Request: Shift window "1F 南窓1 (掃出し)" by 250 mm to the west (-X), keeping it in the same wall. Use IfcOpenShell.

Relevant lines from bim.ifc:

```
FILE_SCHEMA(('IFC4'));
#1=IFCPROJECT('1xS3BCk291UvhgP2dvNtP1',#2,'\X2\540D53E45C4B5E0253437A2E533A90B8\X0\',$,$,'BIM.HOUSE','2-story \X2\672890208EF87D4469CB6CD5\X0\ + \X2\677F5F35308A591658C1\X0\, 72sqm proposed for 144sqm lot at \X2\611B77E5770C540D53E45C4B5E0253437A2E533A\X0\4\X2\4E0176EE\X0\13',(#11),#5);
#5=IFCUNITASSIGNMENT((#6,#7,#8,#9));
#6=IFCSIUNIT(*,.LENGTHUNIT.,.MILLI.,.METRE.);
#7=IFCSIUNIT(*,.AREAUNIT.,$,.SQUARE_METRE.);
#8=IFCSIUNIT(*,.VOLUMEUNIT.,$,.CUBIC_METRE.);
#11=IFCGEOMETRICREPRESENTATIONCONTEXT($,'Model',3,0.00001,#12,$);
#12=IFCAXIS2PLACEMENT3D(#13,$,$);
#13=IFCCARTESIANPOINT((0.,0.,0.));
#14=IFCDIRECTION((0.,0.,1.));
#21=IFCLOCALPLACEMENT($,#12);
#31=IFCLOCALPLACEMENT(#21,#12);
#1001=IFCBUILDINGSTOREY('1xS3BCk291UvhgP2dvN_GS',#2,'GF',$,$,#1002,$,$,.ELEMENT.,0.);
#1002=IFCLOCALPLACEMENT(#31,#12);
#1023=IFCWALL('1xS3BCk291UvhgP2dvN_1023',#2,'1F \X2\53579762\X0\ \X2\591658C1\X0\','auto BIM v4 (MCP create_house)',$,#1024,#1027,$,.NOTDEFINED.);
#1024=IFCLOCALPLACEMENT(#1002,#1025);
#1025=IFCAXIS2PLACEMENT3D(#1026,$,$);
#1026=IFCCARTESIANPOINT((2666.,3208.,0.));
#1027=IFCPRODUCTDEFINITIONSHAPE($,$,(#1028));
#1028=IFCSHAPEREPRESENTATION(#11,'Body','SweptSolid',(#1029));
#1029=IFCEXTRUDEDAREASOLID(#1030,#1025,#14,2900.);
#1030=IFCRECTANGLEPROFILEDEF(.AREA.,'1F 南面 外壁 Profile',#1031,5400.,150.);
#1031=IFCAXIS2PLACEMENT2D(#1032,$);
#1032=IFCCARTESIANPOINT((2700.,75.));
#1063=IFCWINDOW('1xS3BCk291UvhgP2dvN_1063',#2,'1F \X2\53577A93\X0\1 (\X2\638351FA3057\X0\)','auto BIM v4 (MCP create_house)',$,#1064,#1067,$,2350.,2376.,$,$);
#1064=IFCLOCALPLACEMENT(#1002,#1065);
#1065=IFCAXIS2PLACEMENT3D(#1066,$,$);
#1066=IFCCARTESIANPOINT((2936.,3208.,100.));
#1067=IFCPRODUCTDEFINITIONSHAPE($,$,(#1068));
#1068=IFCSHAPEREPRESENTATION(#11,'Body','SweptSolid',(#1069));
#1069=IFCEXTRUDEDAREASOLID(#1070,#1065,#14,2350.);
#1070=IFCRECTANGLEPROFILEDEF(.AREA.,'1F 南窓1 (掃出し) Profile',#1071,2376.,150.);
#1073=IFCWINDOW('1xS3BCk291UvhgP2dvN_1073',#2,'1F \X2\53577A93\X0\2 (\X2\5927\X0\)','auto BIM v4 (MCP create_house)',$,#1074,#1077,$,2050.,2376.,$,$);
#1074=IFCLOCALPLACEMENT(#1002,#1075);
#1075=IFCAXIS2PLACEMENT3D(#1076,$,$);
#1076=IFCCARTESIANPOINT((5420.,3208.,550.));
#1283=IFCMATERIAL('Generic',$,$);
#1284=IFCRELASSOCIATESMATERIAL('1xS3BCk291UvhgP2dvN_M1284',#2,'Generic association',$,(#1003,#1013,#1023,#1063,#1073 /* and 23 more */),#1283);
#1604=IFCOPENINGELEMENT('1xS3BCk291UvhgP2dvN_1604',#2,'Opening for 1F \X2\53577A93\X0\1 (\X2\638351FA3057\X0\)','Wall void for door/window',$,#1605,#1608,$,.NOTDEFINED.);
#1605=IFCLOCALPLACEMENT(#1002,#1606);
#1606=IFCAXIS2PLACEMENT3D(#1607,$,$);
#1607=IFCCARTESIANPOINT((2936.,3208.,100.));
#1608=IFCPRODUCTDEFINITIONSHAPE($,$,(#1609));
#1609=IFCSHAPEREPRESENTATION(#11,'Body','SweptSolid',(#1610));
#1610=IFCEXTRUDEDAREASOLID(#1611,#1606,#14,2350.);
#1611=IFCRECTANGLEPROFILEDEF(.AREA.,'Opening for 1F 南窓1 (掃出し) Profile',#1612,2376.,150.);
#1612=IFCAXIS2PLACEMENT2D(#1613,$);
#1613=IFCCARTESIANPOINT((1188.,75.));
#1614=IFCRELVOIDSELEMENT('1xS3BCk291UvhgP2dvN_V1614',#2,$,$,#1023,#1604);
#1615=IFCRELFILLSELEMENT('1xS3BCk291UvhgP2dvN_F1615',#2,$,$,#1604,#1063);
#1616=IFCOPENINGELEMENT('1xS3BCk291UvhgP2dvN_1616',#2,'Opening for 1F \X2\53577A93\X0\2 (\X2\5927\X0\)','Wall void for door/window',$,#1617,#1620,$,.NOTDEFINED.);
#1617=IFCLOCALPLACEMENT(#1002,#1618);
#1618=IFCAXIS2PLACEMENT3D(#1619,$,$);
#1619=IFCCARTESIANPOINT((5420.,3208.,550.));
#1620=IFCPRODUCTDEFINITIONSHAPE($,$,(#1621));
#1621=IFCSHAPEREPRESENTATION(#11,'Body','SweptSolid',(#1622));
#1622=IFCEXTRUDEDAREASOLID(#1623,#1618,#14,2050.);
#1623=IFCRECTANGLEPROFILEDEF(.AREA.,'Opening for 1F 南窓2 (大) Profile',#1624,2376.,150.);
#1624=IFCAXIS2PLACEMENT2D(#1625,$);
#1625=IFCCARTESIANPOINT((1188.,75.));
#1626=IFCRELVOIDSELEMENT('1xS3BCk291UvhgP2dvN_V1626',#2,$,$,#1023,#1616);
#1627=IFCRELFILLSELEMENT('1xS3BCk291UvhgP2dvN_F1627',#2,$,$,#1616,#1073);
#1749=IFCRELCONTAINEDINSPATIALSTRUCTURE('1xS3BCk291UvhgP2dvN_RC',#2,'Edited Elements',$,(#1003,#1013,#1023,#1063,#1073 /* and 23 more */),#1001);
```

```python
import ifcopenshell
import ifcopenshell.api.geometry
import ifcopenshell.util.placement
import ifcopenshell.util.unit

model = ifcopenshell.open("bim.ifc")
unit_scale = ifcopenshell.util.unit.calculate_unit_scale(model)

window = model.by_id(1063)
opening = window.FillsVoids[0].RelatingOpeningElement
wall = opening.VoidsElements[0].RelatingBuildingElement

wall_matrix = ifcopenshell.util.placement.get_local_placement(wall.ObjectPlacement)
shift = wall_matrix[:3, 0] * -0.25 / unit_scale
before = ifcopenshell.util.placement.get_local_placement(window.ObjectPlacement)[:3, 3].copy()

# The window is not placed relative to its opening, so move both.
for product in (opening, window):
    matrix = ifcopenshell.util.placement.get_local_placement(product.ObjectPlacement)
    matrix[:3, 3] += shift
    ifcopenshell.api.geometry.edit_object_placement(model, product=product, matrix=matrix, is_si=False)

after = ifcopenshell.util.placement.get_local_placement(window.ObjectPlacement)[:3, 3]
print("window moved by", (after - before).round(3) + 0.0)

model.write("bim_edited.ifc")
```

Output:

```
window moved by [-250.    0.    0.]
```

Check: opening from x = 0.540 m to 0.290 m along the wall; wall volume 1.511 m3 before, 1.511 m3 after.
